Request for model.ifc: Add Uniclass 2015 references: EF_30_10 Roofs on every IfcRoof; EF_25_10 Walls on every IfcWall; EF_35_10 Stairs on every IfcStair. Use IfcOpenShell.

First a look at what the model holds.

```python
import ifcopenshell

model = ifcopenshell.open("model.ifc")
print(model.schema)
print("classifications:", [c.Name for c in model.by_type("IfcClassification")])
for ifc_class in ("IfcDoor", "IfcRoof", "IfcStair", "IfcWall", "IfcWindow"):
    print(ifc_class, len(model.by_type(ifc_class)))
```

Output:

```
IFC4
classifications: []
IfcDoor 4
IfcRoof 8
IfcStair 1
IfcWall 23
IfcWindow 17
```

```python
import ifcopenshell
import ifcopenshell.api.classification

model = ifcopenshell.open("model.ifc")

system = ifcopenshell.api.classification.add_classification(model, classification="Uniclass 2015")

codes = {
    "IfcRoof": ("EF_30_10", "Roofs"),
    "IfcWall": ("EF_25_10", "Walls"),
    "IfcStair": ("EF_35_10", "Stairs"),
}
for ifc_class, (code, name) in codes.items():
    products = model.by_type(ifc_class)
    ifcopenshell.api.classification.add_reference(
        model, products=products, classification=system, identification=code, name=name
    )
    print(code, len(products))

model.write("model_v2.ifc")
```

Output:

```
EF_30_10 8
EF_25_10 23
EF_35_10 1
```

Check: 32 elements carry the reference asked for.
